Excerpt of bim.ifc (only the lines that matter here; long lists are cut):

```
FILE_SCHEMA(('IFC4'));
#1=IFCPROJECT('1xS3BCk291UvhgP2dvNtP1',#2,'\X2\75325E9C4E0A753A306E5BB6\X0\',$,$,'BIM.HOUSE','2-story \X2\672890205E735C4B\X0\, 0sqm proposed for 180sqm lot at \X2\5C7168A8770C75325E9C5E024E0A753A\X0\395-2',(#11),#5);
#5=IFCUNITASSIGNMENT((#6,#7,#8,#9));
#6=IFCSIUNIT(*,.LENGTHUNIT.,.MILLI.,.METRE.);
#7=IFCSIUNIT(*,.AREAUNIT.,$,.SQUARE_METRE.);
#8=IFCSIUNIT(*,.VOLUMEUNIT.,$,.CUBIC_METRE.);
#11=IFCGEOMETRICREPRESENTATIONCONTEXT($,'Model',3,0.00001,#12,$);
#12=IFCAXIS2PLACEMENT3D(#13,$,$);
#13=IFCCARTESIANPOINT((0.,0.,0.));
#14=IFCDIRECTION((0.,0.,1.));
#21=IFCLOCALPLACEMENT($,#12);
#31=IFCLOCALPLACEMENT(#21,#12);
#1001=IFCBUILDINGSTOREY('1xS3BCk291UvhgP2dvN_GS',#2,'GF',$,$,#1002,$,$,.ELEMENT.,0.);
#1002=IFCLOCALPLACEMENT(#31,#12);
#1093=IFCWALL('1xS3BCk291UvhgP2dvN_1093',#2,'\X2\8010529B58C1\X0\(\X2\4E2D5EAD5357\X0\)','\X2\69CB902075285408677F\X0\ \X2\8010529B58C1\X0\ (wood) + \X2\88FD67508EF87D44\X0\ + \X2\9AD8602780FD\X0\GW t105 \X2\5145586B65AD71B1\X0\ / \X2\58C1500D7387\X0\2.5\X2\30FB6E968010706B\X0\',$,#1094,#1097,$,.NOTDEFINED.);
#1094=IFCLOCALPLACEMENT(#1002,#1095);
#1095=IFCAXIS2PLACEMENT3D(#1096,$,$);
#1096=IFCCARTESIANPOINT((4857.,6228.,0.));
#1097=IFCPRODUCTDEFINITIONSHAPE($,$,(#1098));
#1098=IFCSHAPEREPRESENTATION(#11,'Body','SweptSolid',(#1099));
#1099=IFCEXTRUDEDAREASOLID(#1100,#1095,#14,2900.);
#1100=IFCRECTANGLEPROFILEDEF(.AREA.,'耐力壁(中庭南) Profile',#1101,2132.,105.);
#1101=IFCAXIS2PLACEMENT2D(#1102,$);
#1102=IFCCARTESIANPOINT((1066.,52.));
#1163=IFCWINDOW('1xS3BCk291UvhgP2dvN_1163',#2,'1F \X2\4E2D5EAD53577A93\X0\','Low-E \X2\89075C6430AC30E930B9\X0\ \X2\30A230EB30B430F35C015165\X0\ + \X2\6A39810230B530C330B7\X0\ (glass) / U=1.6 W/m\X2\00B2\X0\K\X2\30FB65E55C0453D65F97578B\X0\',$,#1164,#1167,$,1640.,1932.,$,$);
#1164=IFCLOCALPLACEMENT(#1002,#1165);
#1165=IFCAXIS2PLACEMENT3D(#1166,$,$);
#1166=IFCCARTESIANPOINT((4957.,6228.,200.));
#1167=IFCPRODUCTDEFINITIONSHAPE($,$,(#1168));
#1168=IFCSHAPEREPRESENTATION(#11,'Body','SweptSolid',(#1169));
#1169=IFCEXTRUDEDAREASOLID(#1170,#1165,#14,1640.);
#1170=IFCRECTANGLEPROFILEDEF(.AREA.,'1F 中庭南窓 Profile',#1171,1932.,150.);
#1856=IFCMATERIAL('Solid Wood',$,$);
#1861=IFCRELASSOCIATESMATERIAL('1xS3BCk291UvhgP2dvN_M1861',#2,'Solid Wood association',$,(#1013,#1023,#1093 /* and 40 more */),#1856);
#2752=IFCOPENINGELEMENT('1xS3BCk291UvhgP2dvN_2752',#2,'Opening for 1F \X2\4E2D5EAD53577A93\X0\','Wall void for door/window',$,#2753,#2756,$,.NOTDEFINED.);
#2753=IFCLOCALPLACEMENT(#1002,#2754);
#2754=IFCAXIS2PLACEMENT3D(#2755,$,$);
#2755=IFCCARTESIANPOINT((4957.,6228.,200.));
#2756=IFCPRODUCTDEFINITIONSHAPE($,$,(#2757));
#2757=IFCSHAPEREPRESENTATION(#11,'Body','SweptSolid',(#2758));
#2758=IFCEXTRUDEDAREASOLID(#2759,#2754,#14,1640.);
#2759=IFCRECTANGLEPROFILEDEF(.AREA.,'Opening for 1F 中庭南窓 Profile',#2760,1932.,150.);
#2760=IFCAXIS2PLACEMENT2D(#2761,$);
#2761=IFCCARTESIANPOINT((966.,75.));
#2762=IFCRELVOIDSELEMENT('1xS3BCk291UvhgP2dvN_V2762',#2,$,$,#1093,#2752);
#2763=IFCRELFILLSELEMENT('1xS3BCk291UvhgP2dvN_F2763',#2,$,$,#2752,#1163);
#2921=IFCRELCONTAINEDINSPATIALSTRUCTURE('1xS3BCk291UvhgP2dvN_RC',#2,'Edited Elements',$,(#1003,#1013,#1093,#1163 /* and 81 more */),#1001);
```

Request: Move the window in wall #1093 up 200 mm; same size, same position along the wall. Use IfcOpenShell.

```python
import numpy as np
import ifcopenshell
import ifcopenshell.api.geometry
import ifcopenshell.util.placement
import ifcopenshell.util.unit

model = ifcopenshell.open("bim.ifc")
unit_scale = ifcopenshell.util.unit.calculate_unit_scale(model)

window = model.by_id(1163)
opening = window.FillsVoids[0].RelatingOpeningElement
dz = 0.2 / unit_scale

shift = np.array([0.0, 0.0, dz])
# The window is not placed relative to its opening, so move both.
for product in (opening, window):
    matrix = ifcopenshell.util.placement.get_local_placement(product.ObjectPlacement)
    matrix[:3, 3] += shift
    ifcopenshell.api.geometry.edit_object_placement(model, product=product, matrix=matrix, is_si=False)

print(f"moved by {dz * unit_scale:+.3f} m")

model.write("bim_edited.ifc")
```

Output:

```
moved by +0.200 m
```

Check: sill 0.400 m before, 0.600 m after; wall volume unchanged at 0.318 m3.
